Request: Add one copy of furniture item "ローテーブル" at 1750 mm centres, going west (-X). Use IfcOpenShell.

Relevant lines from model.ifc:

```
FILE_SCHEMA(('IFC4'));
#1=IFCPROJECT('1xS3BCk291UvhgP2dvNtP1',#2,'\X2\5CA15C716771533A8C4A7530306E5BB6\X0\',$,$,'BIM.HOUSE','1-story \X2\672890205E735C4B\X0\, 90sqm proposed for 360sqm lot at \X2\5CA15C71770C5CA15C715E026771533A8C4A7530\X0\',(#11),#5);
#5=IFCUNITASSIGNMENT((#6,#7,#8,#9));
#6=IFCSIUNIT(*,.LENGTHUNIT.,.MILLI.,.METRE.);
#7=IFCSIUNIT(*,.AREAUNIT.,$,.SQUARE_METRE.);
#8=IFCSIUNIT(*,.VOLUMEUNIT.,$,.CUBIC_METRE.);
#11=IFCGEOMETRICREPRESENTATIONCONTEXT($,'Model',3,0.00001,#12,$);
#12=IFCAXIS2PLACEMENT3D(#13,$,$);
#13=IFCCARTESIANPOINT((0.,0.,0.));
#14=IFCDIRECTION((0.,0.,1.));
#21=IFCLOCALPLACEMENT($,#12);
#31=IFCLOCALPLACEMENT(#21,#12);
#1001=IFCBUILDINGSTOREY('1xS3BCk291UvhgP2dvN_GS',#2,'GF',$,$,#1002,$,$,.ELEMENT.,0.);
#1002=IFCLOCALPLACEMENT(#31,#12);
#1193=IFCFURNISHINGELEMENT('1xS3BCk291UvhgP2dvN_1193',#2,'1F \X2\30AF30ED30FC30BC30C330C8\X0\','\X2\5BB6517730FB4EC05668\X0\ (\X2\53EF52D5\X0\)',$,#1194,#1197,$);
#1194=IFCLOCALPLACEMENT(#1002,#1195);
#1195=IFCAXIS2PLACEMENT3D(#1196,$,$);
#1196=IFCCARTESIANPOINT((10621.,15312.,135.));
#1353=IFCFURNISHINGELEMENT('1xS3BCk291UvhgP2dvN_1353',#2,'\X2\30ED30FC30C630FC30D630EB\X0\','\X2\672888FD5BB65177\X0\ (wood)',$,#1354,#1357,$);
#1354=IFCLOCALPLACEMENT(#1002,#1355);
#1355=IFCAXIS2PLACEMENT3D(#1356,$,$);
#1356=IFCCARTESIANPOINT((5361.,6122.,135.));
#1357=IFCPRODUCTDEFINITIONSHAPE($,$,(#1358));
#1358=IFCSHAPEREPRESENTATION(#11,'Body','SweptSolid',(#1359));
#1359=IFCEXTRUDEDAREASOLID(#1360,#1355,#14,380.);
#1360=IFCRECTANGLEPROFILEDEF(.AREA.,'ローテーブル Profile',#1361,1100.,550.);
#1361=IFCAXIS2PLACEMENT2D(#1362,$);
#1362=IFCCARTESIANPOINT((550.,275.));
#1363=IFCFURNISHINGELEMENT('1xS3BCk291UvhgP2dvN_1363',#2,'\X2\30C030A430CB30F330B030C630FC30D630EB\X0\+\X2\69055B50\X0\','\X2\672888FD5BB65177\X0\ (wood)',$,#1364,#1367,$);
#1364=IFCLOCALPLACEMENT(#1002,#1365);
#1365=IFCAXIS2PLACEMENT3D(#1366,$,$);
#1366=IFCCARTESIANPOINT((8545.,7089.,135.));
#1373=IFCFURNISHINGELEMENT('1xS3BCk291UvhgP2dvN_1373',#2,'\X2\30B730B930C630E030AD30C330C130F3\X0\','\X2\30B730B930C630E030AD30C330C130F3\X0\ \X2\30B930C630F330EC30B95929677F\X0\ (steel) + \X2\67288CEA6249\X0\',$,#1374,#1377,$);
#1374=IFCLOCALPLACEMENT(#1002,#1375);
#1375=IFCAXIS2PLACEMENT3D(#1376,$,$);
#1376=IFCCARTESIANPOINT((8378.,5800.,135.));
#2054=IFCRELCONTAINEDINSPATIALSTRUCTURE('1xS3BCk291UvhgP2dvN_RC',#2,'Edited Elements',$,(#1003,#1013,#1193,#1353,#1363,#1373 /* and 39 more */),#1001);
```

```python
import numpy as np
import ifcopenshell
import ifcopenshell.api.geometry
import ifcopenshell.api.root
import ifcopenshell.util.element
import ifcopenshell.util.placement
import ifcopenshell.util.unit

model = ifcopenshell.open("model.ifc")
unit_scale = ifcopenshell.util.unit.calculate_unit_scale(model)


def reuse_history(source, copy):
    """copy_class also copies each property set's owner history, people and application; keep the originals."""
    for rel in copy.IsDefinedBy:
        if rel.is_a("IfcRelDefinesByProperties") and (history := rel.RelatingPropertyDefinition.OwnerHistory):
            rel.RelatingPropertyDefinition.OwnerHistory = source.OwnerHistory
            ifcopenshell.util.element.remove_deep2(model, history)


source = model.by_guid("1xS3BCk291UvhgP2dvN_1353")
base = ifcopenshell.util.placement.get_local_placement(source.ObjectPlacement)
step = np.array([-1.0, 0.0, 0.0]) * 1.75 / unit_scale

for i in range(1, 2):
    copy = ifcopenshell.api.root.copy_class(model, product=source)
    copy.Representation = ifcopenshell.util.element.copy_deep(
        model, source.Representation, exclude=["IfcGeometricRepresentationContext", "IfcRepresentationMap"]
    )
    reuse_history(source, copy)
    matrix = base.copy()
    matrix[:3, 3] += i * step
    print("added at", matrix[:3, 3].round(3) + 0.0)
    ifcopenshell.api.geometry.edit_object_placement(model, product=copy, matrix=matrix, is_si=False)

model.write("model-out.ifc")
```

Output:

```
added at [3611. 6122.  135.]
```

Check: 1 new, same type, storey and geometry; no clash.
